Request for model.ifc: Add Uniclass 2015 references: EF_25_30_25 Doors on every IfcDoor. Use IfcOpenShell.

First a look at what the model holds.

```python
import ifcopenshell

model = ifcopenshell.open("model.ifc")
print(model.schema)
print("classifications:", [c.Name for c in model.by_type("IfcClassification")])
for ifc_class in ("IfcDoor", "IfcRoof", "IfcStair", "IfcWall", "IfcWindow"):
    print(ifc_class, len(model.by_type(ifc_class)))
```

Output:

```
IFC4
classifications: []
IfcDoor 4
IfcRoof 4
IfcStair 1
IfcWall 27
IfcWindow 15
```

```python
import ifcopenshell
import ifcopenshell.api.classification

model = ifcopenshell.open("model.ifc")

system = ifcopenshell.api.classification.add_classification(model, classification="Uniclass 2015")

codes = {
    "IfcDoor": ("EF_25_30_25", "Doors"),
}
for ifc_class, (code, name) in codes.items():
    products = model.by_type(ifc_class)
    ifcopenshell.api.classification.add_reference(
        model, products=products, classification=system, identification=code, name=name
    )
    print(code, len(products))

model.write("model_v2.ifc")
```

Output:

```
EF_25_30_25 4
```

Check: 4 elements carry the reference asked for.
